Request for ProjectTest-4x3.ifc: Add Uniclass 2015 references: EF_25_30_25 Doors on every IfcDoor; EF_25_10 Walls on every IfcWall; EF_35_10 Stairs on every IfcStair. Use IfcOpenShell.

First a look at what the model holds.

```python
import ifcopenshell

model = ifcopenshell.open("ProjectTest-4x3.ifc")
print(model.schema)
print("classifications:", [c.Name for c in model.by_type("IfcClassification")])
for ifc_class in ("IfcDoor", "IfcRoof", "IfcStair", "IfcWall", "IfcWindow"):
    print(ifc_class, len(model.by_type(ifc_class)))
```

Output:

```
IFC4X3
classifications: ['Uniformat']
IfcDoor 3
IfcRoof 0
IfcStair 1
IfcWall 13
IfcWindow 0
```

```python
import ifcopenshell
import ifcopenshell.api.classification

model = ifcopenshell.open("ProjectTest-4x3.ifc")

system = ifcopenshell.api.classification.add_classification(model, classification="Uniclass 2015")

codes = {
    "IfcDoor": ("EF_25_30_25", "Doors"),
    "IfcWall": ("EF_25_10", "Walls"),
    "IfcStair": ("EF_35_10", "Stairs"),
}
for ifc_class, (code, name) in codes.items():
    products = model.by_type(ifc_class)
    ifcopenshell.api.classification.add_reference(
        model, products=products, classification=system, identification=code, name=name
    )
    print(code, len(products))

model.write("ProjectTest-4x3_rev.ifc")
```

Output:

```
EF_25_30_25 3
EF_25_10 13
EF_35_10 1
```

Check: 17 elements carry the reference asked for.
